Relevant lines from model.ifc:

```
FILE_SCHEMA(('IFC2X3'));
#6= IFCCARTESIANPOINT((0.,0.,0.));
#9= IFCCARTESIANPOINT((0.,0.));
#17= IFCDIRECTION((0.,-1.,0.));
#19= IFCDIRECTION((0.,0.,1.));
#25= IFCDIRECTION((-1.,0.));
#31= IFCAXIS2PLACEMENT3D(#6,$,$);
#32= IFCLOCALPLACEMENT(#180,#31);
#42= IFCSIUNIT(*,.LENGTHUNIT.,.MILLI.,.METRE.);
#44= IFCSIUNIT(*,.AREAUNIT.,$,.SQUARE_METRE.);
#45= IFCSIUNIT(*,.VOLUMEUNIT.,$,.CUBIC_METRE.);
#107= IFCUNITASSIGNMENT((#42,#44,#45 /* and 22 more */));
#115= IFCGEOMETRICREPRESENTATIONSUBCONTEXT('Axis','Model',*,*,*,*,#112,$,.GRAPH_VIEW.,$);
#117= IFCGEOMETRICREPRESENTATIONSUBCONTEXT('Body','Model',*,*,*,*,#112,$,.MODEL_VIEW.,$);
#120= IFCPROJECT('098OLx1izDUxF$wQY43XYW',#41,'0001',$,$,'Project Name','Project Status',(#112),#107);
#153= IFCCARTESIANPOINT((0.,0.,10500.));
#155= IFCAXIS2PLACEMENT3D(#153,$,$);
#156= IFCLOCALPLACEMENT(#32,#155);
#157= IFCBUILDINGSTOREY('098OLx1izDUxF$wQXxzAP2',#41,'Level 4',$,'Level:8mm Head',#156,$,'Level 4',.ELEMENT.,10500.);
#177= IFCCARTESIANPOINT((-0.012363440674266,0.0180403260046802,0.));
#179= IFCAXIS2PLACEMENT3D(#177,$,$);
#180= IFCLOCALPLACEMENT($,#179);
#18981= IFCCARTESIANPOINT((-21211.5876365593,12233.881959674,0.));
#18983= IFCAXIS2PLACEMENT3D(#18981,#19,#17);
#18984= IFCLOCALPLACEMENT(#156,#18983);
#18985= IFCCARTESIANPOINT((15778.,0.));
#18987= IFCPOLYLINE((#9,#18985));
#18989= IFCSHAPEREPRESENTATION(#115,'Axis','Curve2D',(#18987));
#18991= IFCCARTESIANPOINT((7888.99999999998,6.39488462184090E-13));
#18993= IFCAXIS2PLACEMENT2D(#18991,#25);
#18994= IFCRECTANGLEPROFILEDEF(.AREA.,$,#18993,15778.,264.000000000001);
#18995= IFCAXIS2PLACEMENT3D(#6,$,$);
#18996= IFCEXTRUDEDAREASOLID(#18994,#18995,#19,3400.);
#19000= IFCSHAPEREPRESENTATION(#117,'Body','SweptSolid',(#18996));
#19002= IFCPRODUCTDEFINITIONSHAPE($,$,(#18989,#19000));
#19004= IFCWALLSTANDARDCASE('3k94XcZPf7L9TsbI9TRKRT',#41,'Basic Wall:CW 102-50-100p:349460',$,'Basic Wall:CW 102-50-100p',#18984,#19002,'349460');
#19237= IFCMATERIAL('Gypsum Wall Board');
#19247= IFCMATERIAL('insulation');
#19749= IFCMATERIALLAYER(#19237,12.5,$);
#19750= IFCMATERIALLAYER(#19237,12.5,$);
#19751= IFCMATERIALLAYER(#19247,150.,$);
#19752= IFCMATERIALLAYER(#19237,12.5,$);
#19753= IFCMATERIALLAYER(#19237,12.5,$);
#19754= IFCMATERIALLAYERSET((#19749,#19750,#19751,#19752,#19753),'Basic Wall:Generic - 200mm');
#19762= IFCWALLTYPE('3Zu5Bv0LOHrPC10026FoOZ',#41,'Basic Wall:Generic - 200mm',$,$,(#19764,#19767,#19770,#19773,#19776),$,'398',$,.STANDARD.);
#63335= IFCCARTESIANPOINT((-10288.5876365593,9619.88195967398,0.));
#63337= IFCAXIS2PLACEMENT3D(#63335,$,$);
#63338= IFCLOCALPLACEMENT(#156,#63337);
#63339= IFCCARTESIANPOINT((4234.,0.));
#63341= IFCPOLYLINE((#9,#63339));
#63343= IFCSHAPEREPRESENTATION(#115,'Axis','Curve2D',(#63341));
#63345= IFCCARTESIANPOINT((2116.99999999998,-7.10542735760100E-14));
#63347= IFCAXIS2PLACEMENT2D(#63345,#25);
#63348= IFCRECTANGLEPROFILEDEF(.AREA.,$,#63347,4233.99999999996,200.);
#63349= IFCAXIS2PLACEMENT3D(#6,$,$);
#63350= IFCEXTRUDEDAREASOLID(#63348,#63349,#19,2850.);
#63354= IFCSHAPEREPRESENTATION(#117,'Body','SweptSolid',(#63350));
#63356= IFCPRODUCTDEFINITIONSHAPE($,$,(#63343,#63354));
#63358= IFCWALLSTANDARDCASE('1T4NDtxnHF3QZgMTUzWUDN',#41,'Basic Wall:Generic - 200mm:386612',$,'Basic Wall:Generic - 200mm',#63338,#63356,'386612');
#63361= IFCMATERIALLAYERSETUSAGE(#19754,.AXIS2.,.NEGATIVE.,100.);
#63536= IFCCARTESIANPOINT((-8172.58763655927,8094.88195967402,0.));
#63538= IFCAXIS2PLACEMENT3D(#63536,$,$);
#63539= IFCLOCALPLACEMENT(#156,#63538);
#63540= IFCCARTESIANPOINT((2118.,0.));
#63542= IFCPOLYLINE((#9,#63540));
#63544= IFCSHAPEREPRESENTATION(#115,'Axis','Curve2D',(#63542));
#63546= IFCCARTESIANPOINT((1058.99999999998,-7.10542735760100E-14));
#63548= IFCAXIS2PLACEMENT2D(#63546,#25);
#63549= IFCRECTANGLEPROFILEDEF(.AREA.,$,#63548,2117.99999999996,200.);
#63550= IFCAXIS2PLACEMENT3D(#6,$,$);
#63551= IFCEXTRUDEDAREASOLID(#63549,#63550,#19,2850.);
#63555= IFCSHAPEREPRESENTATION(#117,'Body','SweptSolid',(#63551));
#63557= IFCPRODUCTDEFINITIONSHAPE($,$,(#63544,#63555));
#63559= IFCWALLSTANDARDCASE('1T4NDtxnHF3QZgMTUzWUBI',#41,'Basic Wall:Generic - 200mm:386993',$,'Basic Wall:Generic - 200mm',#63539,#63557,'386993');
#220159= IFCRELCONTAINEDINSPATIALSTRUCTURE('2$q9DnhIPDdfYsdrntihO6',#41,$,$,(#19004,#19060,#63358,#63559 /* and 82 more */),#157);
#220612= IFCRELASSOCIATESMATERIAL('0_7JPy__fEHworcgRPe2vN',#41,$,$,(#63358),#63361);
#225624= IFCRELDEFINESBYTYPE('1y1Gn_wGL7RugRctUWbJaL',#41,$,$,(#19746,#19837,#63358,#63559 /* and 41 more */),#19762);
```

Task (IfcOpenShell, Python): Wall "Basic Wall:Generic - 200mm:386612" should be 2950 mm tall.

```python
import ifcopenshell
import ifcopenshell.geom
import ifcopenshell.util.representation
import ifcopenshell.util.shape

model = ifcopenshell.open("model.ifc")
settings = ifcopenshell.geom.settings()


def volume(element):
    """Net volume in cubic metres, openings subtracted."""
    shape = ifcopenshell.geom.create_shape(settings, element)
    return ifcopenshell.util.shape.get_volume(shape.geometry)


wall = model.by_id(63358)
before = volume(wall)

body = ifcopenshell.util.representation.get_representation(wall, "Model", "Body")
solid = body.Items[0]
old_height = solid.Depth
solid.Depth = 2950.0
after = volume(wall)

print(f"height {old_height:g} -> {solid.Depth:g}, volume {before:.3f} -> {after:.3f} m3")

model.write("model_edited.ifc")
```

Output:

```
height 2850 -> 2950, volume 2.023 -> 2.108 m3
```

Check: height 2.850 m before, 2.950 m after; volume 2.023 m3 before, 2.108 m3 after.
